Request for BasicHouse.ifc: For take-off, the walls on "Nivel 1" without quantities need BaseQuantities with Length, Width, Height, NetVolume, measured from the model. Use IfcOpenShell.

First a look at what the model holds.

```python
import ifcopenshell
import ifcopenshell.util.element
import ifcopenshell.util.unit

model = ifcopenshell.open("BasicHouse.ifc")
print(model.schema)
for unit_type in ("LENGTHUNIT", "AREAUNIT", "VOLUMEUNIT"):
    print(unit_type, ifcopenshell.util.unit.calculate_unit_scale(model, unit_type))
storey = next(s for s in model.by_type("IfcBuildingStorey") if s.Name == "Nivel 1")
walls = [e for e in ifcopenshell.util.element.get_decomposition(storey) if e.is_a("IfcWall")]
for e in sorted(walls, key=lambda e: e.id()):
    print(e.id(), e.is_a(), e.Name, list(ifcopenshell.util.element.get_psets(e, qtos_only=True)), sep=" | ")
```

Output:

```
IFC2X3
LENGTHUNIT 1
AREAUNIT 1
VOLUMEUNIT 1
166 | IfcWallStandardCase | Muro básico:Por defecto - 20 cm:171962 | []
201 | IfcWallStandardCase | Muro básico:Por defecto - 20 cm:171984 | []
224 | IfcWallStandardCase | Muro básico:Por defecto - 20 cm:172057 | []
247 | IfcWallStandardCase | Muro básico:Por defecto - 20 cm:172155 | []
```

```python
import ifcopenshell
import ifcopenshell.api.pset
import ifcopenshell.geom
import ifcopenshell.util.element
import ifcopenshell.util.shape
import ifcopenshell.util.unit

model = ifcopenshell.open("BasicHouse.ifc")
unit_scale = ifcopenshell.util.unit.calculate_unit_scale(model)
volume_scale = ifcopenshell.util.unit.calculate_unit_scale(model, "VOLUMEUNIT")
settings = ifcopenshell.geom.settings()

storey = next(s for s in model.by_type("IfcBuildingStorey") if s.Name == "Nivel 1")
walls = [e for e in ifcopenshell.util.element.get_decomposition(storey) if e.is_a("IfcWall")]

for e in sorted(walls, key=lambda e: e.id()):
    if ifcopenshell.util.element.get_psets(e, qtos_only=True, should_inherit=False):
        continue
    # Geometry comes back in metres, in the element's own axes.
    shape = ifcopenshell.geom.create_shape(settings, e)
    values = {
        "Length": ifcopenshell.util.shape.get_x(shape.geometry) / unit_scale,
        "Width": ifcopenshell.util.shape.get_y(shape.geometry) / unit_scale,
        "Height": ifcopenshell.util.shape.get_z(shape.geometry) / unit_scale,
        "NetVolume": ifcopenshell.util.shape.get_volume(shape.geometry) / volume_scale,
    }
    qto = ifcopenshell.api.pset.add_qto(model, product=e, name="BaseQuantities")
    ifcopenshell.api.pset.edit_qto(model, qto=qto, properties=values)
    print(e.id(), {k: round(v, 3) for k, v in values.items()})

model.write("BasicHouse_updated.ifc")
```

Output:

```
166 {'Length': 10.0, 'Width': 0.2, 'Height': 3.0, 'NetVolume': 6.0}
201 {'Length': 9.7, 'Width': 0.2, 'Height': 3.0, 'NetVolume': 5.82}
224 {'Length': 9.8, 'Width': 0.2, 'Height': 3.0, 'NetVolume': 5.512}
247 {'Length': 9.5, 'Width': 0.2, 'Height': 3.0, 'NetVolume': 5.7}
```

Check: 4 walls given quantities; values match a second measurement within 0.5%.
